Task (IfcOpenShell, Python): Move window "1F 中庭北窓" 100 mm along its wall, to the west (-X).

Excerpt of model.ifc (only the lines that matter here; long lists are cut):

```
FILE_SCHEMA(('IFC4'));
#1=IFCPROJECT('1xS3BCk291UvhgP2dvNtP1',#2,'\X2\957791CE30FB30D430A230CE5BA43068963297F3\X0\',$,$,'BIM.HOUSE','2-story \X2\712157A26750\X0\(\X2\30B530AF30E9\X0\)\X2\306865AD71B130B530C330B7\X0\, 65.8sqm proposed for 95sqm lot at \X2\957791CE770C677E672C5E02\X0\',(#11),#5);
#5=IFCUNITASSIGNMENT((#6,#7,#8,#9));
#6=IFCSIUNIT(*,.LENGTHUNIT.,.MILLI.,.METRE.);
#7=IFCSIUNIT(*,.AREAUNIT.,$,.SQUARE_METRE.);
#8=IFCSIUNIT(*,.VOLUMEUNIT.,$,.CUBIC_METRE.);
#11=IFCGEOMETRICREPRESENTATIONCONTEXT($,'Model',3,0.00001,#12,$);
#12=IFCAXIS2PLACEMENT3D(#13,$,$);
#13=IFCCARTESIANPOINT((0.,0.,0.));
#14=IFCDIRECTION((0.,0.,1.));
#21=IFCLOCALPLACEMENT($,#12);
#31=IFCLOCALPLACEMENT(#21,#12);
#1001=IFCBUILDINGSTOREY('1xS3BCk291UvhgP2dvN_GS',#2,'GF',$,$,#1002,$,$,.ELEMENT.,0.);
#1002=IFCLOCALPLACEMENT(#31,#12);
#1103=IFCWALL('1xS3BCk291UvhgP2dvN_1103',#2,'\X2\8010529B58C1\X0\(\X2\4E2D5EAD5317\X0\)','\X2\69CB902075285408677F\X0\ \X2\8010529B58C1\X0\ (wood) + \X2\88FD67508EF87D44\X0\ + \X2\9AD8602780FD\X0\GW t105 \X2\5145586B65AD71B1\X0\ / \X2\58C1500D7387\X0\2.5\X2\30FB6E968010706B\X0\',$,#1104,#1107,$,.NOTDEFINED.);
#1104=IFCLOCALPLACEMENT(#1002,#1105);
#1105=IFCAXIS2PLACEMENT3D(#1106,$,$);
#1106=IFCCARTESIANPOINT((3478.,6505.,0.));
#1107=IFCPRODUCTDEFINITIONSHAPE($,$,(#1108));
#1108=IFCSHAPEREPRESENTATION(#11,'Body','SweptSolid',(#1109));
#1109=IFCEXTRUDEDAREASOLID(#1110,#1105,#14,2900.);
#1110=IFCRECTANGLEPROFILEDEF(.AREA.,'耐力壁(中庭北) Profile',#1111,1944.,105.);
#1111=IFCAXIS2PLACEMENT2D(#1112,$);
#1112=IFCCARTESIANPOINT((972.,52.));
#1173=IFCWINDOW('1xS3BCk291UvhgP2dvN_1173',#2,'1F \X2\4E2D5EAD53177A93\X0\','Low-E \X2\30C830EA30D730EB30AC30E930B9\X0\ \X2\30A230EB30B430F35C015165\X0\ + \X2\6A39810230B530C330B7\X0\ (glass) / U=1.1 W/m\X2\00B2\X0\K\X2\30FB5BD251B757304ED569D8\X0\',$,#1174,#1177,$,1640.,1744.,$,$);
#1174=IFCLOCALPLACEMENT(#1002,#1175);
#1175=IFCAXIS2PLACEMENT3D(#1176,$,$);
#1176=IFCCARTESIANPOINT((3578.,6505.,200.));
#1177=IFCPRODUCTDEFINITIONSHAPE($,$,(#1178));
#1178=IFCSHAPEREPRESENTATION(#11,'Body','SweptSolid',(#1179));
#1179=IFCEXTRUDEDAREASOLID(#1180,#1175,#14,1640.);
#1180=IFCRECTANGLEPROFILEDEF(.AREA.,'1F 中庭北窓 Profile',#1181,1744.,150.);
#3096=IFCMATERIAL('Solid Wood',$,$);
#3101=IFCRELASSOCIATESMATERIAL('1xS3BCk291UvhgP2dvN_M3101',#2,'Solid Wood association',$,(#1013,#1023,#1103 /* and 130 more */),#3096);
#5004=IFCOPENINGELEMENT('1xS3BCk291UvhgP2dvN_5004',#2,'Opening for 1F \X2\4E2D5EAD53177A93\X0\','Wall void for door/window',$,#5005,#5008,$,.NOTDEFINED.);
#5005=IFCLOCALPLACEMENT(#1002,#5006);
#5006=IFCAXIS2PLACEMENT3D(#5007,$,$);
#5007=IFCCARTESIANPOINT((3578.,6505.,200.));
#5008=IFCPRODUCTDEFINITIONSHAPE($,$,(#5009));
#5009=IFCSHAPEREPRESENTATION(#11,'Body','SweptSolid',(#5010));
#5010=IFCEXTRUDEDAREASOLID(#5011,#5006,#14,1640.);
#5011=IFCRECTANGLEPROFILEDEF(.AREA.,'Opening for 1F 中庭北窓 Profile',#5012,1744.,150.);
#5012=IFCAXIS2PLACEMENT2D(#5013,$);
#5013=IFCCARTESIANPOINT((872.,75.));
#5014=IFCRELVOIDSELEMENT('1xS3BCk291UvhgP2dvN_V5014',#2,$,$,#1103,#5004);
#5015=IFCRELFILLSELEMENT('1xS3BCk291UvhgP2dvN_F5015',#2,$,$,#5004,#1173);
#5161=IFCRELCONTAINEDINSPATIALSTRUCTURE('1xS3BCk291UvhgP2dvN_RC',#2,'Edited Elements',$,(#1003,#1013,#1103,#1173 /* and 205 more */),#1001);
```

```python
import ifcopenshell
import ifcopenshell.api.geometry
import ifcopenshell.util.placement
import ifcopenshell.util.unit

model = ifcopenshell.open("model.ifc")
unit_scale = ifcopenshell.util.unit.calculate_unit_scale(model)

window = model.by_guid("1xS3BCk291UvhgP2dvN_1173")
opening = window.FillsVoids[0].RelatingOpeningElement
wall = opening.VoidsElements[0].RelatingBuildingElement

wall_matrix = ifcopenshell.util.placement.get_local_placement(wall.ObjectPlacement)
shift = wall_matrix[:3, 0] * -0.1 / unit_scale
before = ifcopenshell.util.placement.get_local_placement(window.ObjectPlacement)[:3, 3].copy()

# The window is not placed relative to its opening, so move both.
for product in (opening, window):
    matrix = ifcopenshell.util.placement.get_local_placement(product.ObjectPlacement)
    matrix[:3, 3] += shift
    ifcopenshell.api.geometry.edit_object_placement(model, product=product, matrix=matrix, is_si=False)

after = ifcopenshell.util.placement.get_local_placement(window.ObjectPlacement)[:3, 3]
print("window moved by", (after - before).round(3) + 0.0)

model.write("model_rev.ifc")
```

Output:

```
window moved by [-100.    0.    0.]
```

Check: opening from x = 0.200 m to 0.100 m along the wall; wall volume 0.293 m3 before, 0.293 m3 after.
